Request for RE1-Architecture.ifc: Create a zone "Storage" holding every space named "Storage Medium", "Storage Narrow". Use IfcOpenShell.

First a look at what the model holds.

```python
import ifcopenshell

model = ifcopenshell.open("RE1-Architecture.ifc")
print(model.schema)
seen = {}
for space in model.by_type("IfcSpace"):
    seen[space.LongName] = seen.get(space.LongName, 0) + 1
for name, count in sorted(seen.items(), key=str):
    print(count, "x", name)
print("zones:", [z.Name for z in model.by_type("IfcZone")][:20])
```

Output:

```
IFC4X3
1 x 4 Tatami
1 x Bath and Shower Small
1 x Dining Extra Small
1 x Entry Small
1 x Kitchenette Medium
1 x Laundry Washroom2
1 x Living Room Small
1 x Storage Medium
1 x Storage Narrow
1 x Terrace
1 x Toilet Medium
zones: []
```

```python
import ifcopenshell
import ifcopenshell.api.group
import ifcopenshell.api.root

model = ifcopenshell.open("RE1-Architecture.ifc")

names = {"Storage Medium", "Storage Narrow"}
spaces = [s for s in model.by_type("IfcSpace") if s.LongName in names]

zone = ifcopenshell.api.root.create_entity(model, ifc_class="IfcZone", name="Storage")
ifcopenshell.api.group.assign_group(model, products=spaces, group=zone)
print(len(spaces), "spaces in", zone.Name)

model.write("RE1-Architecture_edited.ifc")
```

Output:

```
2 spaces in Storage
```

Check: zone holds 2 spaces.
